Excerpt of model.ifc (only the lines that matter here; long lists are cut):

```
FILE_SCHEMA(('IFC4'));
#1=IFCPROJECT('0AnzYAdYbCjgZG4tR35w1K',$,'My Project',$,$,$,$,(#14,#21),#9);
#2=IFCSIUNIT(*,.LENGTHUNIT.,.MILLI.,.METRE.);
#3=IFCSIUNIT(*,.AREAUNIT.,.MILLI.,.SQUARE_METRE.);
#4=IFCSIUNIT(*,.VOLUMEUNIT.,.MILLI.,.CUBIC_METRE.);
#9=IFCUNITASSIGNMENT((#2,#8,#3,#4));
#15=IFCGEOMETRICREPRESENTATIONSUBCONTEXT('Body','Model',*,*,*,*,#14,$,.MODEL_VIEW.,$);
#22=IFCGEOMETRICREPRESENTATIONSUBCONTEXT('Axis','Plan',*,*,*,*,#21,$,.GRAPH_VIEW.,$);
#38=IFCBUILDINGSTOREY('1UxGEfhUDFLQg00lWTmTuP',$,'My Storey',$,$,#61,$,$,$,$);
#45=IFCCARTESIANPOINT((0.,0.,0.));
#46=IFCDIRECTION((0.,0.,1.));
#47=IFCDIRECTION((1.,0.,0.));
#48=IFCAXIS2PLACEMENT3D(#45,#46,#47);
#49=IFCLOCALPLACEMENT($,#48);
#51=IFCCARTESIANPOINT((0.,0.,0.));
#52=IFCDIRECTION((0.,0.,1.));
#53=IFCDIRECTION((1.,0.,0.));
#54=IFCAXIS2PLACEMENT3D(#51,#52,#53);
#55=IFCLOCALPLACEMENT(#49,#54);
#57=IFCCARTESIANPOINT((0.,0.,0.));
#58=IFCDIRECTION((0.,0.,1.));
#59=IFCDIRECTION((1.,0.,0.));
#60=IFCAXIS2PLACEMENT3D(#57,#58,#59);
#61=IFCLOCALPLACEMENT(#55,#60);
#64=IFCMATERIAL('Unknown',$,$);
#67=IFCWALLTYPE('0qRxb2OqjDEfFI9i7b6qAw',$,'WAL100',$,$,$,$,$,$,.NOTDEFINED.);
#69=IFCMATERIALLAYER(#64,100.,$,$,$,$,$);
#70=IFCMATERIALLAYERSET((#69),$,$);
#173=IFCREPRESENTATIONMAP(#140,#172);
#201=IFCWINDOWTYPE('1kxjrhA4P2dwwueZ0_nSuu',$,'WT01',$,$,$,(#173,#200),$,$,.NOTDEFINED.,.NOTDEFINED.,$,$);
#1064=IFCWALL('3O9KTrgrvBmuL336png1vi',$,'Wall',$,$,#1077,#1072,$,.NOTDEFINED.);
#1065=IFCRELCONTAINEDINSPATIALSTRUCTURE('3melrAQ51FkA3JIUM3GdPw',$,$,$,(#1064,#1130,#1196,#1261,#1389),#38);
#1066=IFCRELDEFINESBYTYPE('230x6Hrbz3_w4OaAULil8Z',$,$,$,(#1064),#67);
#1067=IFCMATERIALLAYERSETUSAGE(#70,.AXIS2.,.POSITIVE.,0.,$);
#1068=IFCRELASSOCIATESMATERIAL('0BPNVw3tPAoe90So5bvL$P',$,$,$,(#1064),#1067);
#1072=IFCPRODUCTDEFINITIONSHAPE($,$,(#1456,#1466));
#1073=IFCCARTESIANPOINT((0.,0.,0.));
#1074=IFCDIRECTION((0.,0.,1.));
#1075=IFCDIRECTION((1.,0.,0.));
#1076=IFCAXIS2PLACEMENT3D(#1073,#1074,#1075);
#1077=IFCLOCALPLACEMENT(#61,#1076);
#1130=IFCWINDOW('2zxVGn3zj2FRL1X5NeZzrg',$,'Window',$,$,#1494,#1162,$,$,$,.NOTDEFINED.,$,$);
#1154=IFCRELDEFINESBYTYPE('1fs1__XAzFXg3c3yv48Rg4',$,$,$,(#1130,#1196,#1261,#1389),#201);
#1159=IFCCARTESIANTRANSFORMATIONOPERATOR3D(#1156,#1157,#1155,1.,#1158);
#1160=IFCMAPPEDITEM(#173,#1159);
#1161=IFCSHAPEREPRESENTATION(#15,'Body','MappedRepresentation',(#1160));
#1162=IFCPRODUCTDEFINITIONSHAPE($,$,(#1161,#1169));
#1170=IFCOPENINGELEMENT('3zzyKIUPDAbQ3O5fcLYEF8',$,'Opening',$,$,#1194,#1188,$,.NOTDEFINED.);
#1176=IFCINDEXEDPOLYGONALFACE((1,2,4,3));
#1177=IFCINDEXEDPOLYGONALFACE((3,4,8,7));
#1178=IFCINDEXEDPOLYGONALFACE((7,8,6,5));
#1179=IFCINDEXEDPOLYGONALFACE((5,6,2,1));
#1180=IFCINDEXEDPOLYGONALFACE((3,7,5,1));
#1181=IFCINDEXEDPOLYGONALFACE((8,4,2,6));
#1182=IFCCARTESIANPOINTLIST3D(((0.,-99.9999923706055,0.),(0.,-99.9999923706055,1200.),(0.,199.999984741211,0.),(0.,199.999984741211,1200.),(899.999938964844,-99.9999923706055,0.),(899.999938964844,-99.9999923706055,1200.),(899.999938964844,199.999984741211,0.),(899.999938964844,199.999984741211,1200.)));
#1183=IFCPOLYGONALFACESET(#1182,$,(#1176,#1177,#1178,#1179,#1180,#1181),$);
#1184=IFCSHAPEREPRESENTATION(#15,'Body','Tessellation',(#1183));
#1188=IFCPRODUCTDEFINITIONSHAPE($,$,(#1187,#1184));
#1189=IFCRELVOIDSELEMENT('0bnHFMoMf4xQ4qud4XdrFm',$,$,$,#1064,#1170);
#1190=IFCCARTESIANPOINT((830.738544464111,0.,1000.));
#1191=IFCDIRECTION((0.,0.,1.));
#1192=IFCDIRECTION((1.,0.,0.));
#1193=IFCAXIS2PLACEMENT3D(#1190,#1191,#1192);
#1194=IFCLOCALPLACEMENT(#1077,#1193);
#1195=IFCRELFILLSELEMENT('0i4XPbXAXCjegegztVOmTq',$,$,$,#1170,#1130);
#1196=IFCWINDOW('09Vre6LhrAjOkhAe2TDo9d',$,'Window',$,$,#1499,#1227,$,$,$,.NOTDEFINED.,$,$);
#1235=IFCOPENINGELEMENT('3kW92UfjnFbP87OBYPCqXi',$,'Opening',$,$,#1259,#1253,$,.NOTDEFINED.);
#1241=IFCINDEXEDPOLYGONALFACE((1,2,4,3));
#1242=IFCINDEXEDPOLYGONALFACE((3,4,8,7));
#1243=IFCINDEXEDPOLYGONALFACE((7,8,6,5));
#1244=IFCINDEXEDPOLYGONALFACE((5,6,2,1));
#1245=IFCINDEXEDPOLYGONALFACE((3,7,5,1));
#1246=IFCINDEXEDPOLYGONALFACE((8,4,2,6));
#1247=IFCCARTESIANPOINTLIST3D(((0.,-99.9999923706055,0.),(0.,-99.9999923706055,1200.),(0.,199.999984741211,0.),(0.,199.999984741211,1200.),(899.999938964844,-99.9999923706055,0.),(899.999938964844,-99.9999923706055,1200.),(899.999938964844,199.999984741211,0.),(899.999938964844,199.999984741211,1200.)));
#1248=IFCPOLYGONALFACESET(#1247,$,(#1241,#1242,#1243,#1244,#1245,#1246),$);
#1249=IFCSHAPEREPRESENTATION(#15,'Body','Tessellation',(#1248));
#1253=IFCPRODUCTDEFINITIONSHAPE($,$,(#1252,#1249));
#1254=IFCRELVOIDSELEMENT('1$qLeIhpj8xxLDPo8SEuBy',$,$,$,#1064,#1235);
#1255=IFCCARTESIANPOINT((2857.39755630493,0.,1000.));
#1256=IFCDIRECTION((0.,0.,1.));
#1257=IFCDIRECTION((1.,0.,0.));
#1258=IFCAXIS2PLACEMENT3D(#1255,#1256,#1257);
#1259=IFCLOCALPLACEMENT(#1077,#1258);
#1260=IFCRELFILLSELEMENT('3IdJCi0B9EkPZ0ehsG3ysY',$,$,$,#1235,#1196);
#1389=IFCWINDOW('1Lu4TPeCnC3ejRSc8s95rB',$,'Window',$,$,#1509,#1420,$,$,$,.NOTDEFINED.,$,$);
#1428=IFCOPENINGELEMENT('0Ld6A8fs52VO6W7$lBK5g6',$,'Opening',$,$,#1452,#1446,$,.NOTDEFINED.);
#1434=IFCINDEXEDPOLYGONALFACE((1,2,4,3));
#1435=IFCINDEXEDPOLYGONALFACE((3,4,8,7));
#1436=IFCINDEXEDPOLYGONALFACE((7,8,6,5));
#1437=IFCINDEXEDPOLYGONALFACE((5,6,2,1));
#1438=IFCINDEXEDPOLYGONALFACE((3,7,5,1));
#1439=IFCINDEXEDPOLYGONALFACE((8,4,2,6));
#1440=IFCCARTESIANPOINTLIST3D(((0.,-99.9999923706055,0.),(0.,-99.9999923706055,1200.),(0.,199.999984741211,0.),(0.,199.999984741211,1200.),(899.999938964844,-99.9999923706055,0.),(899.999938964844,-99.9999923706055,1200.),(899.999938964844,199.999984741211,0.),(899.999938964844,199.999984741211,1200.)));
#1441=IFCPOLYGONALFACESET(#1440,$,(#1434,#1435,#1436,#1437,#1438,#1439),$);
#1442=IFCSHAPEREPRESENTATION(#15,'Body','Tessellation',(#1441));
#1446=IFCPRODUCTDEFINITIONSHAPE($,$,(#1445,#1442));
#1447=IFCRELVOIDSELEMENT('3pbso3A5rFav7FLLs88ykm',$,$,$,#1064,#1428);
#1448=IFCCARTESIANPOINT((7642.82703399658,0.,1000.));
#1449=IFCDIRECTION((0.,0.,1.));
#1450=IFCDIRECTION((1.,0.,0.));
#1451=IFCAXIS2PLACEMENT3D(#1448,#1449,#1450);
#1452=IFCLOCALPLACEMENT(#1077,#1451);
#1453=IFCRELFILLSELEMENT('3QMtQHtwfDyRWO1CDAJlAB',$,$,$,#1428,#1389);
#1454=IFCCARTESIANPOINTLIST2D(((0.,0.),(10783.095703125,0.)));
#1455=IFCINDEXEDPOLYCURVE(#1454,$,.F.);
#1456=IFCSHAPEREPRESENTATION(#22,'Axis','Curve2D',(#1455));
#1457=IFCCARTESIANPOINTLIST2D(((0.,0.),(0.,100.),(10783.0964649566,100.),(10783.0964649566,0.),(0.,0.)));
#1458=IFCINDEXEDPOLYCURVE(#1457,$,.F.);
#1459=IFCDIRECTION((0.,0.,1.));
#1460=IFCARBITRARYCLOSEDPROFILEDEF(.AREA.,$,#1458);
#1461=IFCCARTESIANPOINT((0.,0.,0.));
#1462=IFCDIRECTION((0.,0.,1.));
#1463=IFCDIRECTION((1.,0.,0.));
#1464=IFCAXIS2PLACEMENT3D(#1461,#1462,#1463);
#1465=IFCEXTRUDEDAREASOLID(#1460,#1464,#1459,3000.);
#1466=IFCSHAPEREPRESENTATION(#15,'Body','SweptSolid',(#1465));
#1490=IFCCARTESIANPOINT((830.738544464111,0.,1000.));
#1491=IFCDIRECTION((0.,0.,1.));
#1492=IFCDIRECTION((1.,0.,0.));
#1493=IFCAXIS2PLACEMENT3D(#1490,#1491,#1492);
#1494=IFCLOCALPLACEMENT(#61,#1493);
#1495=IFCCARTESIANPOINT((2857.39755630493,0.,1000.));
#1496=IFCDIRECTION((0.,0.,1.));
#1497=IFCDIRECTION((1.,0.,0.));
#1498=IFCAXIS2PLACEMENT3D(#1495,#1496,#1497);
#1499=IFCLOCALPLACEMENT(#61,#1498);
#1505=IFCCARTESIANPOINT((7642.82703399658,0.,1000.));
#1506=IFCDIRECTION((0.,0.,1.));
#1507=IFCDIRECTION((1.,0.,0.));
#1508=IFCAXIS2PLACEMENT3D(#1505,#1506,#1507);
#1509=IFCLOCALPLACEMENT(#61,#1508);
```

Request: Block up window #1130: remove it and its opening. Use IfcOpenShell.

```python
import ifcopenshell
import ifcopenshell.api.feature
import ifcopenshell.api.root
import ifcopenshell.geom
import ifcopenshell.util.shape

model = ifcopenshell.open("model.ifc")
settings = ifcopenshell.geom.settings()


def volume(element):
    """Net volume in cubic metres, openings subtracted."""
    shape = ifcopenshell.geom.create_shape(settings, element)
    return ifcopenshell.util.shape.get_volume(shape.geometry)


window = model.by_guid("2zxVGn3zj2FRL1X5NeZzrg")
opening = window.FillsVoids[0].RelatingOpeningElement
wall = opening.VoidsElements[0].RelatingBuildingElement
before = volume(wall)

ifcopenshell.api.root.remove_product(model, product=window)
ifcopenshell.api.feature.remove_feature(model, feature=opening)

after = volume(wall)

print(f"wall volume {before:.3f} -> {after:.3f} m3")

model.write("model_edited.ifc")
```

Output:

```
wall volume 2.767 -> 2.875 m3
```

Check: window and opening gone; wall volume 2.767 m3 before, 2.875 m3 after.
